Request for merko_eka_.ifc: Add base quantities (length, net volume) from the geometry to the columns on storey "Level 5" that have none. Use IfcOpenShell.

First a look at what the model holds.

```python
import ifcopenshell
import ifcopenshell.util.element
import ifcopenshell.util.unit

model = ifcopenshell.open("merko_eka_.ifc")
print(model.schema)
for unit_type in ("LENGTHUNIT", "AREAUNIT", "VOLUMEUNIT"):
    print(unit_type, ifcopenshell.util.unit.calculate_unit_scale(model, unit_type))
storey = next(s for s in model.by_type("IfcBuildingStorey") if s.Name == "Level 5")
columns = [e for e in ifcopenshell.util.element.get_decomposition(storey) if e.is_a("IfcColumn")]
for e in sorted(columns, key=lambda e: e.id()):
    print(e.id(), e.is_a(), e.Name, list(ifcopenshell.util.element.get_psets(e, qtos_only=True)), sep=" | ")
```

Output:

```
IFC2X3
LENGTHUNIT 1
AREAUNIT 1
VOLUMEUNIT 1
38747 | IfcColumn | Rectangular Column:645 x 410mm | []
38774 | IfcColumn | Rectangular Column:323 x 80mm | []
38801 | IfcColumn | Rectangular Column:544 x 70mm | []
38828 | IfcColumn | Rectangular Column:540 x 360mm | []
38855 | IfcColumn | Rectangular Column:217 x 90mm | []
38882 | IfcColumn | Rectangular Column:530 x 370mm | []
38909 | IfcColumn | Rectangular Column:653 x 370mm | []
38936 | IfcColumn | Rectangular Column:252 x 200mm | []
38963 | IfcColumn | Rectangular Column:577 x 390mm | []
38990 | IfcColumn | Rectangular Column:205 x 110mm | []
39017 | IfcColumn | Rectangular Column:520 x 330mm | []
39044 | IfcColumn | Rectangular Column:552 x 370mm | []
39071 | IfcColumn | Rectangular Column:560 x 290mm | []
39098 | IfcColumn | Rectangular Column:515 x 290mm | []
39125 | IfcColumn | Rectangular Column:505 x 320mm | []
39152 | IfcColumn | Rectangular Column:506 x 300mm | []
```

```python
import ifcopenshell
import ifcopenshell.api.pset
import ifcopenshell.geom
import ifcopenshell.util.element
import ifcopenshell.util.shape
import ifcopenshell.util.unit

model = ifcopenshell.open("merko_eka_.ifc")
unit_scale = ifcopenshell.util.unit.calculate_unit_scale(model)
volume_scale = ifcopenshell.util.unit.calculate_unit_scale(model, "VOLUMEUNIT")
settings = ifcopenshell.geom.settings()

storey = next(s for s in model.by_type("IfcBuildingStorey") if s.Name == "Level 5")
columns = [e for e in ifcopenshell.util.element.get_decomposition(storey) if e.is_a("IfcColumn")]

for e in sorted(columns, key=lambda e: e.id()):
    if ifcopenshell.util.element.get_psets(e, qtos_only=True, should_inherit=False):
        continue
    # Geometry comes back in metres, in the element's own axes.
    shape = ifcopenshell.geom.create_shape(settings, e)
    values = {
        "Length": ifcopenshell.util.shape.get_z(shape.geometry) / unit_scale,
        "NetVolume": ifcopenshell.util.shape.get_volume(shape.geometry) / volume_scale,
    }
    qto = ifcopenshell.api.pset.add_qto(model, product=e, name="BaseQuantities")
    ifcopenshell.api.pset.edit_qto(model, qto=qto, properties=values)
    print(e.id(), {k: round(v, 3) for k, v in values.items()})

model.write("merko_eka__edited.ifc")
```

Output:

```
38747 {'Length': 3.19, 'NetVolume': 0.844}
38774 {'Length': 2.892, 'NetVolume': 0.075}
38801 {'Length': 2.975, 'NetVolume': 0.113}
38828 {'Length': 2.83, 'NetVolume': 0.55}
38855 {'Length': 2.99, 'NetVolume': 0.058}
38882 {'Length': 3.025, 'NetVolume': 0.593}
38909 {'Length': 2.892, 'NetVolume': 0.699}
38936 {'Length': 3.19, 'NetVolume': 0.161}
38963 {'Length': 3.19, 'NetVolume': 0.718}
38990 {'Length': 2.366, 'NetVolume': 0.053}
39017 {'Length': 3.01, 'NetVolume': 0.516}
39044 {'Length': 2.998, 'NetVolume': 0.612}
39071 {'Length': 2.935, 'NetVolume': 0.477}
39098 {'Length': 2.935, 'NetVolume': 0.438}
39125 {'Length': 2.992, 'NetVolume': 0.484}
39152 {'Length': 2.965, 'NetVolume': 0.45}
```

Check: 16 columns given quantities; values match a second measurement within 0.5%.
